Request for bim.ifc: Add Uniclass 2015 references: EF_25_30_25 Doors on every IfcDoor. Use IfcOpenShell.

First a look at what the model holds.

```python
import ifcopenshell

model = ifcopenshell.open("bim.ifc")
print(model.schema)
print("classifications:", [c.Name for c in model.by_type("IfcClassification")])
for ifc_class in ("IfcDoor", "IfcRoof", "IfcStair", "IfcWall", "IfcWindow"):
    print(ifc_class, len(model.by_type(ifc_class)))
```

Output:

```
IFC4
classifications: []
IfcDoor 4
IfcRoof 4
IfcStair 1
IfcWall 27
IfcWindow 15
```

```python
import ifcopenshell
import ifcopenshell.api.classification

model = ifcopenshell.open("bim.ifc")

system = ifcopenshell.api.classification.add_classification(model, classification="Uniclass 2015")

codes = {
    "IfcDoor": ("EF_25_30_25", "Doors"),
}
for ifc_class, (code, name) in codes.items():
    products = model.by_type(ifc_class)
    ifcopenshell.api.classification.add_reference(
        model, products=products, classification=system, identification=code, name=name
    )
    print(code, len(products))

model.write("bim-out.ifc")
```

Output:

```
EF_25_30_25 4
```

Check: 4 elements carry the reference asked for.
